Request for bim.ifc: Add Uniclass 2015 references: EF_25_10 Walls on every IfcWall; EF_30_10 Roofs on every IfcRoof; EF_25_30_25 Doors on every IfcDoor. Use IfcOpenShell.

First a look at what the model holds.

```python
import ifcopenshell

model = ifcopenshell.open("bim.ifc")
print(model.schema)
print("classifications:", [c.Name for c in model.by_type("IfcClassification")])
for ifc_class in ("IfcDoor", "IfcRoof", "IfcStair", "IfcWall", "IfcWindow"):
    print(ifc_class, len(model.by_type(ifc_class)))
```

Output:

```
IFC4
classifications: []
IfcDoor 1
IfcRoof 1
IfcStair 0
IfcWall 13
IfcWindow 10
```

```python
import ifcopenshell
import ifcopenshell.api.classification

model = ifcopenshell.open("bim.ifc")

system = ifcopenshell.api.classification.add_classification(model, classification="Uniclass 2015")

codes = {
    "IfcWall": ("EF_25_10", "Walls"),
    "IfcRoof": ("EF_30_10", "Roofs"),
    "IfcDoor": ("EF_25_30_25", "Doors"),
}
for ifc_class, (code, name) in codes.items():
    products = model.by_type(ifc_class)
    ifcopenshell.api.classification.add_reference(
        model, products=products, classification=system, identification=code, name=name
    )
    print(code, len(products))

model.write("bim_v2.ifc")
```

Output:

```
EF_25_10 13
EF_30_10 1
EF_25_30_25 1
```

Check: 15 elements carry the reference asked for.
